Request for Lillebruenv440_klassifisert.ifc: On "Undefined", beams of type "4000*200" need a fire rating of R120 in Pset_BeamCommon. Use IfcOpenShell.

First a look at what the model holds.

```python
import ifcopenshell
import ifcopenshell.util.element

model = ifcopenshell.open("Lillebruenv440_klassifisert.ifc")
print(model.schema)
storey = next(s for s in model.by_type("IfcBuildingStorey") if s.Name == "Undefined")
beams = [e for e in ifcopenshell.util.element.get_decomposition(storey) if e.is_a("IfcBeam")]
seen = {}
for e in beams:
    element_type = ifcopenshell.util.element.get_type(e)
    key = (element_type.Name if element_type != e and element_type else None, ifcopenshell.util.element.get_pset(e, "Pset_BeamCommon", "FireRating"))
    seen[key] = seen.get(key, 0) + 1
for (name, value), count in sorted(seen.items(), key=str):
    print(count, "x", name, "|", value)
```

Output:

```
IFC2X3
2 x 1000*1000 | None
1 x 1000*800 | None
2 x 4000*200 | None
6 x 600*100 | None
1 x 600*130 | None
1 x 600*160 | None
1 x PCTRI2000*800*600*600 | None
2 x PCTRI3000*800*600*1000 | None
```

```python
import ifcopenshell
import ifcopenshell.api.pset
import ifcopenshell.util.element

model = ifcopenshell.open("Lillebruenv440_klassifisert.ifc")

storey = next(s for s in model.by_type("IfcBuildingStorey") if s.Name == "Undefined")
beams = [e for e in ifcopenshell.util.element.get_decomposition(storey) if e.is_a("IfcBeam")]

count = 0
for e in beams:
    element_type = ifcopenshell.util.element.get_type(e)
    if element_type in (None, e) or element_type.Name != "4000*200":
        continue
    found = ifcopenshell.util.element.get_pset(e, "Pset_BeamCommon", should_inherit=False)
    if found:
        pset = model.by_id(found["id"])
        if len(ifcopenshell.util.element.get_elements_by_pset(pset)) > 1:
            pset = ifcopenshell.api.pset.unshare_pset(model, products=[e], pset=pset)[0]
    else:
        pset = ifcopenshell.api.pset.add_pset(model, product=e, name="Pset_BeamCommon")
    ifcopenshell.api.pset.edit_pset(model, pset=pset, properties={"FireRating": "R120"})
    count += 1

print(count, "beams updated")

model.write("Lillebruenv440_klassifisert_rev.ifc")
```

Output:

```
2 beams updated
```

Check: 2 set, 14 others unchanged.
